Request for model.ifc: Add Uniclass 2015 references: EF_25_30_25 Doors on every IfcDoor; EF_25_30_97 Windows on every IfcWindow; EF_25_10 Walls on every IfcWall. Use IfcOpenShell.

First a look at what the model holds.

```python
import ifcopenshell

model = ifcopenshell.open("model.ifc")
print(model.schema)
print("classifications:", [c.Name for c in model.by_type("IfcClassification")])
for ifc_class in ("IfcDoor", "IfcRoof", "IfcStair", "IfcWall", "IfcWindow"):
    print(ifc_class, len(model.by_type(ifc_class)))
```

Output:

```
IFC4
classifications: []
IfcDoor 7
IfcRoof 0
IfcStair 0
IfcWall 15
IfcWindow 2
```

```python
import ifcopenshell
import ifcopenshell.api.classification

model = ifcopenshell.open("model.ifc")

system = ifcopenshell.api.classification.add_classification(model, classification="Uniclass 2015")

codes = {
    "IfcDoor": ("EF_25_30_25", "Doors"),
    "IfcWindow": ("EF_25_30_97", "Windows"),
    "IfcWall": ("EF_25_10", "Walls"),
}
for ifc_class, (code, name) in codes.items():
    products = model.by_type(ifc_class)
    ifcopenshell.api.classification.add_reference(
        model, products=products, classification=system, identification=code, name=name
    )
    print(code, len(products))

model.write("model_edited.ifc")
```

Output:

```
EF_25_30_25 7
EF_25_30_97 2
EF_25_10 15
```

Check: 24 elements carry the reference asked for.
